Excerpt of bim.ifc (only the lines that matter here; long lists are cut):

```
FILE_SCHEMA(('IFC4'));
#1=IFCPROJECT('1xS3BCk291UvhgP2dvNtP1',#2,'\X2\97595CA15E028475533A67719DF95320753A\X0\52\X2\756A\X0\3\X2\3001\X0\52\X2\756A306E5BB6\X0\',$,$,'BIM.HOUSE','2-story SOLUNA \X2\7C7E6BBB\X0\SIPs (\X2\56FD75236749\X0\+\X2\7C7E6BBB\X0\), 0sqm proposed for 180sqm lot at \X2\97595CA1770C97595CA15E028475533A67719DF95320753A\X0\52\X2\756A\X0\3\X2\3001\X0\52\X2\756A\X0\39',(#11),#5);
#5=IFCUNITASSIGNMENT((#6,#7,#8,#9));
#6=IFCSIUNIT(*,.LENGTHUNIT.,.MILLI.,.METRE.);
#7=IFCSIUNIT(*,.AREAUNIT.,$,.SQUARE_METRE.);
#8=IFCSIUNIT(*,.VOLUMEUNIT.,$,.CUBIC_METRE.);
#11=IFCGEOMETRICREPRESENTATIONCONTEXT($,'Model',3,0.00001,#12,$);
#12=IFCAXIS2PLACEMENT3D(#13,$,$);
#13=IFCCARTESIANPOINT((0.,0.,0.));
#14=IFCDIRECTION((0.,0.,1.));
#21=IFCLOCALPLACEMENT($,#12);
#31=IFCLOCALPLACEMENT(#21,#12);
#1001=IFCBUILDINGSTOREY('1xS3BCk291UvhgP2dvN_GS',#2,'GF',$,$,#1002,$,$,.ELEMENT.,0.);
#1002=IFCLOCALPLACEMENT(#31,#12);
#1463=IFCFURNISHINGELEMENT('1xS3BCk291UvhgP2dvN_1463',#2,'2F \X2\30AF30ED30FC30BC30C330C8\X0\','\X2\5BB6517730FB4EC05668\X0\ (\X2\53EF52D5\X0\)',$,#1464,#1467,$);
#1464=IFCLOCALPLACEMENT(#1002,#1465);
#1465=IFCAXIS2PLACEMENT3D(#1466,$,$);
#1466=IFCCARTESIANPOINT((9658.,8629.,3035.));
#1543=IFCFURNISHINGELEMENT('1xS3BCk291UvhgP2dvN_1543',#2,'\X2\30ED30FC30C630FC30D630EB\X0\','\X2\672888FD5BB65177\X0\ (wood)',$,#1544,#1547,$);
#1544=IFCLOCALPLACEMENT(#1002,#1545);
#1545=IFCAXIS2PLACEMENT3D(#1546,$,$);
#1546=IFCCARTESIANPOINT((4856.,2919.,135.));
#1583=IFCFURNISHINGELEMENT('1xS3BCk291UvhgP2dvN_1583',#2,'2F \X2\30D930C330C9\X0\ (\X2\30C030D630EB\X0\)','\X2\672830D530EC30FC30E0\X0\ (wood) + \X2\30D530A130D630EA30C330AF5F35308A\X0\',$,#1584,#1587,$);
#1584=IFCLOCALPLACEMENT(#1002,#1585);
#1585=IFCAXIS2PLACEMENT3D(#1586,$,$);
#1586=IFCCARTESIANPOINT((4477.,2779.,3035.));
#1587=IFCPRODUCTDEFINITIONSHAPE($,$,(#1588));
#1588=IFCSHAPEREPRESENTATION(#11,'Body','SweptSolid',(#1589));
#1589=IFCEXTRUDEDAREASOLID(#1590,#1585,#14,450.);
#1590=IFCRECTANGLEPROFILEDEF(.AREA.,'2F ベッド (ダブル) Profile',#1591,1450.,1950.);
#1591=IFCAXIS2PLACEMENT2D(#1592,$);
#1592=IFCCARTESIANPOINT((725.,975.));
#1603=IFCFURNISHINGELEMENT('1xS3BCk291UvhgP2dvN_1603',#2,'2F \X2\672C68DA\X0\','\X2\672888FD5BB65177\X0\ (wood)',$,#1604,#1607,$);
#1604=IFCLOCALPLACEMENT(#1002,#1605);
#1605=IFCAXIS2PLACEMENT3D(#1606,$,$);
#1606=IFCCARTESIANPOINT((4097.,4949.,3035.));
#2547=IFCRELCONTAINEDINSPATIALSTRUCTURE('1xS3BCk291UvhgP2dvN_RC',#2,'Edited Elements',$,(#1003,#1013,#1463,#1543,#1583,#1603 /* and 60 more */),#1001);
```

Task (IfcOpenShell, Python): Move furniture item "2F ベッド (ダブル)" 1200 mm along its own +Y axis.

```python
import ifcopenshell
import ifcopenshell.api.geometry
import ifcopenshell.util.placement
import ifcopenshell.util.unit

model = ifcopenshell.open("bim.ifc")
unit_scale = ifcopenshell.util.unit.calculate_unit_scale(model)

item = model.by_guid("1xS3BCk291UvhgP2dvN_1583")
matrix = ifcopenshell.util.placement.get_local_placement(item.ObjectPlacement)
matrix[:3, 3] += matrix[:3, 1] * 1.2 / unit_scale
ifcopenshell.api.geometry.edit_object_placement(model, product=item, matrix=matrix, is_si=False)

print(ifcopenshell.util.placement.get_local_placement(item.ObjectPlacement).round(3) + 0.0)

model.write("bim_rev.ifc")
```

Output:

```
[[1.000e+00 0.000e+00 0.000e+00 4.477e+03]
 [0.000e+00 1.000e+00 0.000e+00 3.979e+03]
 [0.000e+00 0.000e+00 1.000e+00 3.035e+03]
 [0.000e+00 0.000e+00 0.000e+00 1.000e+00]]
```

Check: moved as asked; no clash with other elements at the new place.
